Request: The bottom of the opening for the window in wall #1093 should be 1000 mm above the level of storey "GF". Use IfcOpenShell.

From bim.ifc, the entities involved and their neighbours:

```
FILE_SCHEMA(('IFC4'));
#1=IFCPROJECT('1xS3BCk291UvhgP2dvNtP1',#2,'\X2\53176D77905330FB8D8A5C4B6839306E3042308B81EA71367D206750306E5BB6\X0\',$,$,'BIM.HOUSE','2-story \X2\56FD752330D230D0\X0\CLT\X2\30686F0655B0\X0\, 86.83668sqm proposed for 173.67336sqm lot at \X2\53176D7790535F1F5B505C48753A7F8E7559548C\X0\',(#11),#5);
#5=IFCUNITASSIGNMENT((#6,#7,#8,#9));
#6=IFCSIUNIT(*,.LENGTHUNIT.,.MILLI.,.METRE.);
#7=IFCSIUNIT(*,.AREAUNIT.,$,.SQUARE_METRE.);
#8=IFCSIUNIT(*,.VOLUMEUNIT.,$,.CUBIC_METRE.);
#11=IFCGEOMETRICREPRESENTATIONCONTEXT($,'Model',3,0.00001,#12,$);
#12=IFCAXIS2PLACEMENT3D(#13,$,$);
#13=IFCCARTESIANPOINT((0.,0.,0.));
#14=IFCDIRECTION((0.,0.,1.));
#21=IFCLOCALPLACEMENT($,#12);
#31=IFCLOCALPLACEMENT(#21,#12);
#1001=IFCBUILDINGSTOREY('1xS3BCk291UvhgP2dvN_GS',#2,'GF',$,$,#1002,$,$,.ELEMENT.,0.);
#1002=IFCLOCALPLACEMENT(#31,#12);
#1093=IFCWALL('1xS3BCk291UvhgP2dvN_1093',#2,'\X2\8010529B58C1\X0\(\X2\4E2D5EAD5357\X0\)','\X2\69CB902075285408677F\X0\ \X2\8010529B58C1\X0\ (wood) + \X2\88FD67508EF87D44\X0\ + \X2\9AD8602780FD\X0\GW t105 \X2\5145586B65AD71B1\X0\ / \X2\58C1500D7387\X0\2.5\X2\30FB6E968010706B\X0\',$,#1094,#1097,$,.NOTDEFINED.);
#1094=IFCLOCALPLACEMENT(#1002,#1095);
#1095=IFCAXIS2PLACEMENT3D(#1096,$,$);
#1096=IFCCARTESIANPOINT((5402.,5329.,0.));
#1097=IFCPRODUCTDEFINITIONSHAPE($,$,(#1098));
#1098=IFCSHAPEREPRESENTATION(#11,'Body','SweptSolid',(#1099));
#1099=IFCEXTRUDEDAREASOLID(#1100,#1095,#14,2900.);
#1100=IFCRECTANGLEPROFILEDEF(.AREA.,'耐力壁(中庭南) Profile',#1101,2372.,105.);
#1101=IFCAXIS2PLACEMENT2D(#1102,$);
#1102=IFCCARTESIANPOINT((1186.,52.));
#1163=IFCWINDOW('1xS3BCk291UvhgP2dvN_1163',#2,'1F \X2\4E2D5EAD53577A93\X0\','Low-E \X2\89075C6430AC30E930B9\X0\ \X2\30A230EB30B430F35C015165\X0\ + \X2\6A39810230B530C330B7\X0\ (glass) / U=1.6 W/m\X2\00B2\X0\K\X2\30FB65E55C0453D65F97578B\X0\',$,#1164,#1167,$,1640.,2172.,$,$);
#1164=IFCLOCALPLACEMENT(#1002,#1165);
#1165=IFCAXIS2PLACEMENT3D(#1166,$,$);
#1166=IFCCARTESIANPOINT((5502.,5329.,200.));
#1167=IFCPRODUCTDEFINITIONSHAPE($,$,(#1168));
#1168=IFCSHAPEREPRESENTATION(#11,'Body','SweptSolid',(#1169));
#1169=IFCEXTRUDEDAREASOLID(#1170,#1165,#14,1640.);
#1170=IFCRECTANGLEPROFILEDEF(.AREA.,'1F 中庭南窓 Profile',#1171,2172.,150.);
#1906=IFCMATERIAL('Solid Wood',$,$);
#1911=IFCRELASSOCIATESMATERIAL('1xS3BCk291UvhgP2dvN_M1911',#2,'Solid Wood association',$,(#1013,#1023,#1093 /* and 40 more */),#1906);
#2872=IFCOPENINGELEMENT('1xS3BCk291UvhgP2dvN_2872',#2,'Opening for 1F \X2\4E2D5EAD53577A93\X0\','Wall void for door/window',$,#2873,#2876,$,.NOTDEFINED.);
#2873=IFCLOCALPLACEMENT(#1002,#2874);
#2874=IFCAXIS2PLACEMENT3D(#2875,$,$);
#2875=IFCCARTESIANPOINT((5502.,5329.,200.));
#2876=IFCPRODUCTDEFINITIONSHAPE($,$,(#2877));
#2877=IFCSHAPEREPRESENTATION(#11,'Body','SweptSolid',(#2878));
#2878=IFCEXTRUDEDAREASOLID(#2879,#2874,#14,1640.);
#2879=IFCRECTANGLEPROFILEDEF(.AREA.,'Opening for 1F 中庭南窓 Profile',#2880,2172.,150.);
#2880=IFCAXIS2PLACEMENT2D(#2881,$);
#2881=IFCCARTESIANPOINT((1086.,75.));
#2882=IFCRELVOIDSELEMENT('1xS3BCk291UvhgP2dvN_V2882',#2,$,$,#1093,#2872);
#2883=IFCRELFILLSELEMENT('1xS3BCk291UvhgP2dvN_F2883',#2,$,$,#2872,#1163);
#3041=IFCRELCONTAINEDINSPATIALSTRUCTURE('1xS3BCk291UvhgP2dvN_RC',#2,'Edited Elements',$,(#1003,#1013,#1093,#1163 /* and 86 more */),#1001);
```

```python
import numpy as np
import ifcopenshell
import ifcopenshell.api.geometry
import ifcopenshell.geom
import ifcopenshell.util.element
import ifcopenshell.util.placement
import ifcopenshell.util.shape
import ifcopenshell.util.unit

model = ifcopenshell.open("bim.ifc")
unit_scale = ifcopenshell.util.unit.calculate_unit_scale(model)

window = model.by_guid("1xS3BCk291UvhgP2dvN_1163")
opening = window.FillsVoids[0].RelatingOpeningElement
storey = ifcopenshell.util.element.get_container(window, ifc_class="IfcBuildingStorey")
level = ifcopenshell.util.placement.get_local_placement(storey.ObjectPlacement)[2, 3]

# The opening's origin need not be at the sill, so measure its lowest point.
shape = ifcopenshell.geom.create_shape(ifcopenshell.geom.settings(), opening)
bottom = ifcopenshell.util.shape.get_shape_bottom_elevation(shape, shape.geometry) / unit_scale
dz = level + 1 / unit_scale - bottom

shift = np.array([0.0, 0.0, dz])
# The window is not placed relative to its opening, so move both.
for product in (opening, window):
    matrix = ifcopenshell.util.placement.get_local_placement(product.ObjectPlacement)
    matrix[:3, 3] += shift
    ifcopenshell.api.geometry.edit_object_placement(model, product=product, matrix=matrix, is_si=False)

print(f"moved by {dz * unit_scale:+.3f} m")

model.write("bim-out.ifc")
```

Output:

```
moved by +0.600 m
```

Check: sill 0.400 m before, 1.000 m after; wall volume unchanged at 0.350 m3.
